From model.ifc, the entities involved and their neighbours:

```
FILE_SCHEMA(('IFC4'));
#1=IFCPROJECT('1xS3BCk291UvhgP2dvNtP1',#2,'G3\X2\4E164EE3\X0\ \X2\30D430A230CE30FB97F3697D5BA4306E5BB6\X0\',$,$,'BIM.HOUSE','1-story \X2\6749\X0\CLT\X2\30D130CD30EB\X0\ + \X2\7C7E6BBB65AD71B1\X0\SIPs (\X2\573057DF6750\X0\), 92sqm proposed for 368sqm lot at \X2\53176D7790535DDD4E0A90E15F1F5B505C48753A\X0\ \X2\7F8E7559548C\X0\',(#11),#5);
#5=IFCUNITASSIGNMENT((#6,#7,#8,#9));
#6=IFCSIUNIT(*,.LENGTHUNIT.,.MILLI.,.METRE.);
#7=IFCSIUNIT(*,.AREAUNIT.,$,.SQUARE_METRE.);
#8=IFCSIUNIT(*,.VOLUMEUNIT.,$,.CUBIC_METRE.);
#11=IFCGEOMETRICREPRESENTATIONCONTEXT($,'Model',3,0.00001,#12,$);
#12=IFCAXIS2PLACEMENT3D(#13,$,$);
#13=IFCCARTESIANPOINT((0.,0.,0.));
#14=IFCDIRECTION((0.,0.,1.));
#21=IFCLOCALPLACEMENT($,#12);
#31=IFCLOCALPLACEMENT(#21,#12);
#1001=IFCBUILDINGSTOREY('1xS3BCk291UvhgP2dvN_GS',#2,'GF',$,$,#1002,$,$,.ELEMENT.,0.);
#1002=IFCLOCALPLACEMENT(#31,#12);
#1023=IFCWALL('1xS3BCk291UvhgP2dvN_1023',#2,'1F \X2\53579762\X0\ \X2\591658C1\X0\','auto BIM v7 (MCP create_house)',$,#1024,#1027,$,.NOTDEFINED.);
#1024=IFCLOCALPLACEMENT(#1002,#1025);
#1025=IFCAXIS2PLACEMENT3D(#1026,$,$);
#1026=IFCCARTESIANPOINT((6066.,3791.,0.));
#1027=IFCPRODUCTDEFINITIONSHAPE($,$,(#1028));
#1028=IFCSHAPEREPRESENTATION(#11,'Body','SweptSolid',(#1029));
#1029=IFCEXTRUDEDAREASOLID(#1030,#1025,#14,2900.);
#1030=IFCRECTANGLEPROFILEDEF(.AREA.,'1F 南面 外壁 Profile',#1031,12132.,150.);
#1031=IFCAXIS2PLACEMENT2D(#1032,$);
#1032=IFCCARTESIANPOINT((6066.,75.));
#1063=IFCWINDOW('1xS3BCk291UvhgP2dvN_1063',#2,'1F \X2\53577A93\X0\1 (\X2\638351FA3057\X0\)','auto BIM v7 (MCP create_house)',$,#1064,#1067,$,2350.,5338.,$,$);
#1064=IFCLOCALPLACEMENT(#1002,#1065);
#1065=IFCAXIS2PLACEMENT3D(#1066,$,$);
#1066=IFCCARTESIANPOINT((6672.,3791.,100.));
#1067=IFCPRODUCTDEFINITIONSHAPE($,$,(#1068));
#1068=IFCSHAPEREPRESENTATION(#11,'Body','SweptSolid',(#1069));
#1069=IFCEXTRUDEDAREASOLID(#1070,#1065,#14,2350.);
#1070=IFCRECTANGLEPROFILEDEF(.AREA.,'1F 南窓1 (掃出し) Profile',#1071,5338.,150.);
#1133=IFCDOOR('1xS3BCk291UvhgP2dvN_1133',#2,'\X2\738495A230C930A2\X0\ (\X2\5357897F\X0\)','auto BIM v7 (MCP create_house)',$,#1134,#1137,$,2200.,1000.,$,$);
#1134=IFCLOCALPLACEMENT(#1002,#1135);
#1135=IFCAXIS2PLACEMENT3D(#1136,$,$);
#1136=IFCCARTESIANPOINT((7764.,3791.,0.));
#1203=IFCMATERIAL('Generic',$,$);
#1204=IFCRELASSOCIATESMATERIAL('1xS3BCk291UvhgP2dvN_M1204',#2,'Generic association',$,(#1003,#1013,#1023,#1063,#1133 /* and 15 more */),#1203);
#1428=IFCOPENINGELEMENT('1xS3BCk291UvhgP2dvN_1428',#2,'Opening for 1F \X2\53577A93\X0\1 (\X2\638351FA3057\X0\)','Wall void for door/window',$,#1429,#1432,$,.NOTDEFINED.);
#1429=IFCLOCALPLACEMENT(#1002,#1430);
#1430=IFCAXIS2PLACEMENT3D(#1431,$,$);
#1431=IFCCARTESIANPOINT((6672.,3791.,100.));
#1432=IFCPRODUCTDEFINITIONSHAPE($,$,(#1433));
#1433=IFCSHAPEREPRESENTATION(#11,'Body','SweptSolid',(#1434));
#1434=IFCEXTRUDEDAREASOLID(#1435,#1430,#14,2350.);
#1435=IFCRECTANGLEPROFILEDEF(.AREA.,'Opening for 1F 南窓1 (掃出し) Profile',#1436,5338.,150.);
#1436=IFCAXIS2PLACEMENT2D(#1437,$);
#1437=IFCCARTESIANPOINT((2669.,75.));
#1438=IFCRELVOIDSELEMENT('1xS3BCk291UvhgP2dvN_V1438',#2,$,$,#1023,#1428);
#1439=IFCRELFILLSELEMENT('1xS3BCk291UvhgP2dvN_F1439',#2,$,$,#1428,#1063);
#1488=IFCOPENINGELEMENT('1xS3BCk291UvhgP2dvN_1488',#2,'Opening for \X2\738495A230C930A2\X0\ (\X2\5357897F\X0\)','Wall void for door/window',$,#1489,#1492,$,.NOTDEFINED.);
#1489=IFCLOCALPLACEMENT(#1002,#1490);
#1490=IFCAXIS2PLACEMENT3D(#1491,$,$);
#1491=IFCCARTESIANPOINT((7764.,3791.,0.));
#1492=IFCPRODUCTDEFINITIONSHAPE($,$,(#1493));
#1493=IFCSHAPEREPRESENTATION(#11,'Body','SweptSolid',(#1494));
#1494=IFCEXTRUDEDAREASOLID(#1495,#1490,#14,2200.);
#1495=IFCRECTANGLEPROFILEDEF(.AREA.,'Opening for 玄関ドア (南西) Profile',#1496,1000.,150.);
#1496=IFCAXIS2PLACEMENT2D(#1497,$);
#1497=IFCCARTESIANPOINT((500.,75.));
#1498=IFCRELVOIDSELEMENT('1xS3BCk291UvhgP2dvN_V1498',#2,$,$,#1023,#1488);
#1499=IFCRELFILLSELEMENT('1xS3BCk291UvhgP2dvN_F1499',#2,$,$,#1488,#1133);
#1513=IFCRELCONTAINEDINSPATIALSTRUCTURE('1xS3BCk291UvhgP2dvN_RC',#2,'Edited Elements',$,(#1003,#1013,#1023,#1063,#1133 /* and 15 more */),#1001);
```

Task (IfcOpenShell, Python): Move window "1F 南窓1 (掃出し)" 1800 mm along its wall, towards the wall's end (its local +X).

```python
import ifcopenshell
import ifcopenshell.api.geometry
import ifcopenshell.util.placement

model = ifcopenshell.open("model.ifc")

window = model.by_id(1063)
opening = window.FillsVoids[0].RelatingOpeningElement
wall = opening.VoidsElements[0].RelatingBuildingElement

wall_matrix = ifcopenshell.util.placement.get_local_placement(wall.ObjectPlacement)
shift = wall_matrix[:3, 0] * 1800.0
before = ifcopenshell.util.placement.get_local_placement(window.ObjectPlacement)[:3, 3].copy()

# The window is not placed relative to its opening, so move both.
for product in (opening, window):
    matrix = ifcopenshell.util.placement.get_local_placement(product.ObjectPlacement)
    matrix[:3, 3] += shift
    ifcopenshell.api.geometry.edit_object_placement(model, product=product, matrix=matrix, is_si=False)

after = ifcopenshell.util.placement.get_local_placement(window.ObjectPlacement)[:3, 3]
print("window moved by", (after - before).round(3) + 0.0)

model.write("model_updated.ifc")
```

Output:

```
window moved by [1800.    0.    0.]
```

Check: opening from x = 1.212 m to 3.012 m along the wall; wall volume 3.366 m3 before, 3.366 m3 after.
